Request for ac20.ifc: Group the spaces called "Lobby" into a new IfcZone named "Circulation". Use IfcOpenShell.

First a look at what the model holds.

```python
import ifcopenshell

model = ifcopenshell.open("ac20.ifc")
print(model.schema)
seen = {}
for space in model.by_type("IfcSpace"):
    seen[space.LongName] = seen.get(space.LongName, 0) + 1
for name, count in sorted(seen.items(), key=str):
    print(count, "x", name)
print("zones:", [z.Name for z in model.by_type("IfcZone")][:20])
```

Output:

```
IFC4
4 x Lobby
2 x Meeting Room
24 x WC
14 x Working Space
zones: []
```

```python
import ifcopenshell
import ifcopenshell.api.group
import ifcopenshell.api.root

model = ifcopenshell.open("ac20.ifc")

names = {"Lobby"}
spaces = [s for s in model.by_type("IfcSpace") if s.LongName in names]

zone = ifcopenshell.api.root.create_entity(model, ifc_class="IfcZone", name="Circulation")
ifcopenshell.api.group.assign_group(model, products=spaces, group=zone)
print(len(spaces), "spaces in", zone.Name)

model.write("ac20_rev.ifc")
```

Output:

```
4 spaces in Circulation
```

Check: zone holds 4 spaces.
